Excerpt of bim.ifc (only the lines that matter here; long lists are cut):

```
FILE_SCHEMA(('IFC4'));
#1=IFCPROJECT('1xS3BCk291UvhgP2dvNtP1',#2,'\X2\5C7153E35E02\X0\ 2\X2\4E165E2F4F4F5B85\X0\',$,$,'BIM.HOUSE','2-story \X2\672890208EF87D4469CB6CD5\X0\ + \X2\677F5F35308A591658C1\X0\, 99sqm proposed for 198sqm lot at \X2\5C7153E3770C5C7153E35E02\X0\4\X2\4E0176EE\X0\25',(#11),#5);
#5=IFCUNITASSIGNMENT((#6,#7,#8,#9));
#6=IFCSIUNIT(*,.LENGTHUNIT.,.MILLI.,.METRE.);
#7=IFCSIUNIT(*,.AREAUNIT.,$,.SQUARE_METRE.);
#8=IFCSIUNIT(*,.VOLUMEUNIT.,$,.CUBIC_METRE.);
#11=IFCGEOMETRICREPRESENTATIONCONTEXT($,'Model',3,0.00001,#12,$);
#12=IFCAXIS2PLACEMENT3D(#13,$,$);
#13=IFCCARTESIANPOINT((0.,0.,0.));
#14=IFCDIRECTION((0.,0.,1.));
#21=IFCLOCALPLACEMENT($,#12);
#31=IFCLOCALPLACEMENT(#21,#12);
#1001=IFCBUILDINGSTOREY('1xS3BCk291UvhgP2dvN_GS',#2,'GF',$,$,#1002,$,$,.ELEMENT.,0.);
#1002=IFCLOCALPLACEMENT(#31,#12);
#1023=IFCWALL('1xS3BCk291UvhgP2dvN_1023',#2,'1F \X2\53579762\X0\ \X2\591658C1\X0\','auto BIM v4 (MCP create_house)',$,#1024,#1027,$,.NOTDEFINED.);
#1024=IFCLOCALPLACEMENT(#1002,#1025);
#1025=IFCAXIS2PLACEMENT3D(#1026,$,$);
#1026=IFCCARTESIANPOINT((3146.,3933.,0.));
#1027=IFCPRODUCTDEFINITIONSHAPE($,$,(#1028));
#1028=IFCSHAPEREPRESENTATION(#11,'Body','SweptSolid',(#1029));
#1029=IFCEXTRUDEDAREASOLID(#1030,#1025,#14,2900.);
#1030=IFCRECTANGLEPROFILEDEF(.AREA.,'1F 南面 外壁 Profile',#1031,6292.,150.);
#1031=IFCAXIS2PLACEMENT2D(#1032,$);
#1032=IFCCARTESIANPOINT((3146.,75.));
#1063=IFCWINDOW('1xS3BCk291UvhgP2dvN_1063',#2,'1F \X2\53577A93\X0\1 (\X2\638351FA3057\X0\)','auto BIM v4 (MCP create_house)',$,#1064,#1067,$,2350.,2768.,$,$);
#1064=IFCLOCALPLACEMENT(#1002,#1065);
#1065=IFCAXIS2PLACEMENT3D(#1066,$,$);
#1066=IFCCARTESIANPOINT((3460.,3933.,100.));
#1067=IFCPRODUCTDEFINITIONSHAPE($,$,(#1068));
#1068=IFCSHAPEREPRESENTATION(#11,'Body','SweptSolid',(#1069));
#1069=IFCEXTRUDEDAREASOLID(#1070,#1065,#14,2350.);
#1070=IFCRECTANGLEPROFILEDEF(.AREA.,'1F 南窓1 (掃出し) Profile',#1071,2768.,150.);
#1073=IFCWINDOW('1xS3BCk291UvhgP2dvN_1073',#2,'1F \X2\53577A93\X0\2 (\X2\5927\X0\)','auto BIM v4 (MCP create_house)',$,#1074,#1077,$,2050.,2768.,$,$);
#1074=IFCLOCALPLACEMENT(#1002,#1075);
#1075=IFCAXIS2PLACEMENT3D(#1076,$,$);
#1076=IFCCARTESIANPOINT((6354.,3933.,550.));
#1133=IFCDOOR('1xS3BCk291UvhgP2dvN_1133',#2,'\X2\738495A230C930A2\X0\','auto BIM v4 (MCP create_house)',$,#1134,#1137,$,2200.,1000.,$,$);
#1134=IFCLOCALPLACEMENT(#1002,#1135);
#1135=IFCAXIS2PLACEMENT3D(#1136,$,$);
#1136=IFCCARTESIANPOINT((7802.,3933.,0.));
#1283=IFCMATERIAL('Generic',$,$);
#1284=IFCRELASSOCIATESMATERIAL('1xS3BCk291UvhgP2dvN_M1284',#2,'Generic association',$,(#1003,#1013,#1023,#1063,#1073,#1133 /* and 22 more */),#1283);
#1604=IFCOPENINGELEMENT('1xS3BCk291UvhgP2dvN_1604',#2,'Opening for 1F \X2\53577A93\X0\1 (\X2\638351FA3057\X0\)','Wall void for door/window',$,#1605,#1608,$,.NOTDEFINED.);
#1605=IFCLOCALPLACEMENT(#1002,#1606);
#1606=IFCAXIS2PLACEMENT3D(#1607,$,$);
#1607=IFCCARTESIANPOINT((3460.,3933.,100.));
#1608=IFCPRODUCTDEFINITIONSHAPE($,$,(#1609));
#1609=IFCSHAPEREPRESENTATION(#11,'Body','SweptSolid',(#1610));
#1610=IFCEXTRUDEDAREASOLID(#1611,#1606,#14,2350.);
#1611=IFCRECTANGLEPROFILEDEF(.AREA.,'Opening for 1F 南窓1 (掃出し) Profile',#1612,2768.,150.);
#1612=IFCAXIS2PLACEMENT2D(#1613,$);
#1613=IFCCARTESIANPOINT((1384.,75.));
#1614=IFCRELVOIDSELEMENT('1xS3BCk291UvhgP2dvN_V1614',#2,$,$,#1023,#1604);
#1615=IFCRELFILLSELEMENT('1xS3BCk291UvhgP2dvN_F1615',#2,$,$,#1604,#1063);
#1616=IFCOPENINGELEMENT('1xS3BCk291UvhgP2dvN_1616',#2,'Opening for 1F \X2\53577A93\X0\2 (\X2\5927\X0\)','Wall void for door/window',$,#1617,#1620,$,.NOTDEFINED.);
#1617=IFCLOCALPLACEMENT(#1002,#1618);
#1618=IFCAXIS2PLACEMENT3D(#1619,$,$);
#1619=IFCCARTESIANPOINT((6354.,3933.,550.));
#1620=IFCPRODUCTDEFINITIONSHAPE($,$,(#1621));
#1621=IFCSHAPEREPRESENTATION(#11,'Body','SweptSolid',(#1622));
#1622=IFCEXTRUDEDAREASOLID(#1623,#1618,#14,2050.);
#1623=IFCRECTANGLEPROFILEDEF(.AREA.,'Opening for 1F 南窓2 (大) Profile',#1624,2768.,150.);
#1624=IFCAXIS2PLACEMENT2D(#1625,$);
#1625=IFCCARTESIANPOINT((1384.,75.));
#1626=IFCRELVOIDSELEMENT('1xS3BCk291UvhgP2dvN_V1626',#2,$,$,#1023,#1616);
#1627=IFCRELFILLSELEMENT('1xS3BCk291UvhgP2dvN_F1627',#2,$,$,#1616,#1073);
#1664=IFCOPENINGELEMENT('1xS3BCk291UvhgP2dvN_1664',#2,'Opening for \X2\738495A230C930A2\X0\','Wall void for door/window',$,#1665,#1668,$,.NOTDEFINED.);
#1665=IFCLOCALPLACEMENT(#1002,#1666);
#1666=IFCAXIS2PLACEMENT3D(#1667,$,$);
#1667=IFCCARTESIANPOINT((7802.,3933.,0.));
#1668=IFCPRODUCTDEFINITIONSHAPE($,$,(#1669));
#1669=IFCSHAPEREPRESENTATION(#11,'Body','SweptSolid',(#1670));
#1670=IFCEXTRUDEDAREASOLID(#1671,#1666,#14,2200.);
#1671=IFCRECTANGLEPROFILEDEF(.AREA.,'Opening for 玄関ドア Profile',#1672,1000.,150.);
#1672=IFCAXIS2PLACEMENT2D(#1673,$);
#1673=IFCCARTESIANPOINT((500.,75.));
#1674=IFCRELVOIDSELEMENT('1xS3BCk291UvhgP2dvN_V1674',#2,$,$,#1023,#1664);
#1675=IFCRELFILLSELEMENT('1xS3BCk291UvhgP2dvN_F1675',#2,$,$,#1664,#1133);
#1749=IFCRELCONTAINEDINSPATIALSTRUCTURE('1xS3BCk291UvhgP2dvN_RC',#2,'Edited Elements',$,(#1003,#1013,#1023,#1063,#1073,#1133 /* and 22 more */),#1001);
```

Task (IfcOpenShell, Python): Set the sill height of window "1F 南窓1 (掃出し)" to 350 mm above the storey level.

```python
import numpy as np
import ifcopenshell
import ifcopenshell.api.geometry
import ifcopenshell.geom
import ifcopenshell.util.element
import ifcopenshell.util.placement
import ifcopenshell.util.shape
import ifcopenshell.util.unit

model = ifcopenshell.open("bim.ifc")
unit_scale = ifcopenshell.util.unit.calculate_unit_scale(model)

window = model.by_guid("1xS3BCk291UvhgP2dvN_1063")
opening = window.FillsVoids[0].RelatingOpeningElement
storey = ifcopenshell.util.element.get_container(window, ifc_class="IfcBuildingStorey")
level = ifcopenshell.util.placement.get_local_placement(storey.ObjectPlacement)[2, 3]

# The opening's origin need not be at the sill, so measure its lowest point.
shape = ifcopenshell.geom.create_shape(ifcopenshell.geom.settings(), opening)
bottom = ifcopenshell.util.shape.get_shape_bottom_elevation(shape, shape.geometry) / unit_scale
dz = level + 0.35 / unit_scale - bottom

shift = np.array([0.0, 0.0, dz])
# The window is not placed relative to its opening, so move both.
for product in (opening, window):
    matrix = ifcopenshell.util.placement.get_local_placement(product.ObjectPlacement)
    matrix[:3, 3] += shift
    ifcopenshell.api.geometry.edit_object_placement(model, product=product, matrix=matrix, is_si=False)

print(f"moved by {dz * unit_scale:+.3f} m")

model.write("bim_edited.ifc")
```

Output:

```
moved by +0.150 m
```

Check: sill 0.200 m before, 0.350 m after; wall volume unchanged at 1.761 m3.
